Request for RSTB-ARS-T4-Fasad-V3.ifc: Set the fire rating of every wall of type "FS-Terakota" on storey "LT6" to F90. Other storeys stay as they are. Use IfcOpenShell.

First a look at what the model holds.

```python
import ifcopenshell
import ifcopenshell.util.element

model = ifcopenshell.open("RSTB-ARS-T4-Fasad-V3.ifc")
print(model.schema)
storey = next(s for s in model.by_type("IfcBuildingStorey") if s.Name == "LT6")
walls = [e for e in ifcopenshell.util.element.get_decomposition(storey) if e.is_a("IfcWall")]
seen = {}
for e in walls:
    element_type = ifcopenshell.util.element.get_type(e)
    key = (element_type.Name if element_type != e and element_type else None, ifcopenshell.util.element.get_pset(e, "Pset_WallCommon", "FireRating"))
    seen[key] = seen.get(key, 0) + 1
for (name, value), count in sorted(seen.items(), key=str):
    print(count, "x", name, "|", value)
```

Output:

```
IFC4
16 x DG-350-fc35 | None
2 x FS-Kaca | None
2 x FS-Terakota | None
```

```python
import ifcopenshell
import ifcopenshell.api.pset
import ifcopenshell.util.element

model = ifcopenshell.open("RSTB-ARS-T4-Fasad-V3.ifc")

storey = next(s for s in model.by_type("IfcBuildingStorey") if s.Name == "LT6")
walls = [e for e in ifcopenshell.util.element.get_decomposition(storey) if e.is_a("IfcWall")]

count = 0
for e in walls:
    element_type = ifcopenshell.util.element.get_type(e)
    if element_type in (None, e) or element_type.Name != "FS-Terakota":
        continue
    # add_pset returns the element's existing set when there is one.
    pset = ifcopenshell.api.pset.add_pset(model, product=e, name="Pset_WallCommon")
    ifcopenshell.api.pset.edit_pset(model, pset=pset, properties={"FireRating": "F90"})
    count += 1

print(count, "walls updated")

model.write("RSTB-ARS-T4-Fasad-V3_edited.ifc")
```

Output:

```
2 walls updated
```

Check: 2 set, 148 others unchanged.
